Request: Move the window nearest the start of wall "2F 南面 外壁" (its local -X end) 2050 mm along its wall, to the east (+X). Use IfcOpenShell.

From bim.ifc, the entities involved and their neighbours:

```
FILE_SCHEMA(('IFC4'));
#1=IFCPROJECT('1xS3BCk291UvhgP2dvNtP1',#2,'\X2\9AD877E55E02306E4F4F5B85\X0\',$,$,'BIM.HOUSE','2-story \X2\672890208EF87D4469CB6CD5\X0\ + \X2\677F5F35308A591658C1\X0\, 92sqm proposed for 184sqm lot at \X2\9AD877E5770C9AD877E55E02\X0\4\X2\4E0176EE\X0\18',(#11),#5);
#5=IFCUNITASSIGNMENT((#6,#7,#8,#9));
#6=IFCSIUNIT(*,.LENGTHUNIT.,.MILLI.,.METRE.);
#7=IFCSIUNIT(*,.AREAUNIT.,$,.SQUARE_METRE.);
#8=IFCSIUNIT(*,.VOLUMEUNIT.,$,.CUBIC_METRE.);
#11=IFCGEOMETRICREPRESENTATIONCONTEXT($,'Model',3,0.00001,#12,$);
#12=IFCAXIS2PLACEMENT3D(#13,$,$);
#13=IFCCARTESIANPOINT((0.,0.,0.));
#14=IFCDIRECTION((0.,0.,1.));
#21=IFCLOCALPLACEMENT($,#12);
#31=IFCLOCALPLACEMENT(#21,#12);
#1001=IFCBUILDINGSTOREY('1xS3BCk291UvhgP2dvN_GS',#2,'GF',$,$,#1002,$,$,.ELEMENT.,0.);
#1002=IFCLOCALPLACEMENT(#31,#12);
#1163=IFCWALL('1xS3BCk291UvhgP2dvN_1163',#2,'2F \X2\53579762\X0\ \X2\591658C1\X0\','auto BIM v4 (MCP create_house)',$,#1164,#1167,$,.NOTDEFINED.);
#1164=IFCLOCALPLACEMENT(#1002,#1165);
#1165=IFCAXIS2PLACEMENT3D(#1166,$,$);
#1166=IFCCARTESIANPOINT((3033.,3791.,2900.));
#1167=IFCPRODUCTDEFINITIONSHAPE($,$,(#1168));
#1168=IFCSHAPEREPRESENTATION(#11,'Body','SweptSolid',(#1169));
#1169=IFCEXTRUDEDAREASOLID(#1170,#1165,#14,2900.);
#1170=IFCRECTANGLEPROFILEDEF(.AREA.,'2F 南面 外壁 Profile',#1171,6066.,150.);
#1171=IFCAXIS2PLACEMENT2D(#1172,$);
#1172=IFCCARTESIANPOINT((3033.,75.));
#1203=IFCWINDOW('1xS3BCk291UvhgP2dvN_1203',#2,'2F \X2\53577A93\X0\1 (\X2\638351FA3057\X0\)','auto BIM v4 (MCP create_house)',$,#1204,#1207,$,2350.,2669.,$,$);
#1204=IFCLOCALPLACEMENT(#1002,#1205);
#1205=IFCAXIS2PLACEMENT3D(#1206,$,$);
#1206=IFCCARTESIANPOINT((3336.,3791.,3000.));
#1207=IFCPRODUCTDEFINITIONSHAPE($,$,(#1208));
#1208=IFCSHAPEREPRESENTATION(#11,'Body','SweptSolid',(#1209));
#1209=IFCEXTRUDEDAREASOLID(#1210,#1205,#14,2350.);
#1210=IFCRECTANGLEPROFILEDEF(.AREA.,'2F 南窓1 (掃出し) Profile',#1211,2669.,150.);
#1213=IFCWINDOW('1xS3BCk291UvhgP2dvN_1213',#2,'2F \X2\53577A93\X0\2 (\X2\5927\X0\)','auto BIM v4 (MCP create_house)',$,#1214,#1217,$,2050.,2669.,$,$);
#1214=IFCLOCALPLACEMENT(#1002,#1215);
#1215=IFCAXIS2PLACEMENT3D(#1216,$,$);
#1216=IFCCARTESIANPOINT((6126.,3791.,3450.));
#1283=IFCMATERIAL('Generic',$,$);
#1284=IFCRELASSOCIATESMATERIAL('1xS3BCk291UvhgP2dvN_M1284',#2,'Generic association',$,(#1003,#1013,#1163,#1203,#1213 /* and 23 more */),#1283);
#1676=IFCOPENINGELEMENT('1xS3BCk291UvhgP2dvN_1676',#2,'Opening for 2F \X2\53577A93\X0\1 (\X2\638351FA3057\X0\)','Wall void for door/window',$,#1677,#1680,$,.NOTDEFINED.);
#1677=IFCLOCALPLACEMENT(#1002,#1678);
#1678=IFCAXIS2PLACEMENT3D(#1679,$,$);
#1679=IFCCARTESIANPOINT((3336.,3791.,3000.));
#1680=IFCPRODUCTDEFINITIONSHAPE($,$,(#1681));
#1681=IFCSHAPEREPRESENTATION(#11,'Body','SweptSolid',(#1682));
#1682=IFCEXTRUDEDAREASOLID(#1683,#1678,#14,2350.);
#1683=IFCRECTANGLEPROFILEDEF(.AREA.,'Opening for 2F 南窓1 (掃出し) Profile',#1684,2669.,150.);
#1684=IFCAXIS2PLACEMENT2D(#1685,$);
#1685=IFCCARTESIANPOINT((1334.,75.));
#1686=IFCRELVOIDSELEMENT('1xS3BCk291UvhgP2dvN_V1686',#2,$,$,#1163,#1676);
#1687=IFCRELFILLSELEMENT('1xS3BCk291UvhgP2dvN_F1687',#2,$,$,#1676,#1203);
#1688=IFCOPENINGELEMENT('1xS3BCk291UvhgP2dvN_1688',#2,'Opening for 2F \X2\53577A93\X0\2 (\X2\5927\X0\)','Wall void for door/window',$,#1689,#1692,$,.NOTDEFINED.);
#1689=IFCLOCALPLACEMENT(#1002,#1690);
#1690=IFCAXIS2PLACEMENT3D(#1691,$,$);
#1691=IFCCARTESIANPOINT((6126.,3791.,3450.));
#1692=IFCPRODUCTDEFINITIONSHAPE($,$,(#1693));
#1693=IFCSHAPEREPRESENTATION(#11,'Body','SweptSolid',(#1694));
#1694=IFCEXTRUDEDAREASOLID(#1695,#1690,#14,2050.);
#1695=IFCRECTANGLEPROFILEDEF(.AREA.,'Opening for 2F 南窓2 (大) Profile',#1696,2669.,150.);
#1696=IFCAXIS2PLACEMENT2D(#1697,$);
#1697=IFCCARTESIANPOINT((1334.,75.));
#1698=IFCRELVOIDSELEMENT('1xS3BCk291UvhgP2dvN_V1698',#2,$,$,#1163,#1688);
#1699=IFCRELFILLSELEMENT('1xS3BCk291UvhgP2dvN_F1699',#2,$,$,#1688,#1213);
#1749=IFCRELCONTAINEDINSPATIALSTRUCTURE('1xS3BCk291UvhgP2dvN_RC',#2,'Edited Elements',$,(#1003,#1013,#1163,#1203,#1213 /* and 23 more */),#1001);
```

```python
import ifcopenshell
import ifcopenshell.api.geometry
import ifcopenshell.util.placement

model = ifcopenshell.open("bim.ifc")

window = model.by_id(1203)
opening = window.FillsVoids[0].RelatingOpeningElement
wall = opening.VoidsElements[0].RelatingBuildingElement

wall_matrix = ifcopenshell.util.placement.get_local_placement(wall.ObjectPlacement)
shift = wall_matrix[:3, 0] * 2050.0
before = ifcopenshell.util.placement.get_local_placement(window.ObjectPlacement)[:3, 3].copy()

# The window is not placed relative to its opening, so move both.
for product in (opening, window):
    matrix = ifcopenshell.util.placement.get_local_placement(product.ObjectPlacement)
    matrix[:3, 3] += shift
    ifcopenshell.api.geometry.edit_object_placement(model, product=product, matrix=matrix, is_si=False)

after = ifcopenshell.util.placement.get_local_placement(window.ObjectPlacement)[:3, 3]
print("window moved by", (after - before).round(3) + 0.0)

model.write("bim_updated.ifc")
```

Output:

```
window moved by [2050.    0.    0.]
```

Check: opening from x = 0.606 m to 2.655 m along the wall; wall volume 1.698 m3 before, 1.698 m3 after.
